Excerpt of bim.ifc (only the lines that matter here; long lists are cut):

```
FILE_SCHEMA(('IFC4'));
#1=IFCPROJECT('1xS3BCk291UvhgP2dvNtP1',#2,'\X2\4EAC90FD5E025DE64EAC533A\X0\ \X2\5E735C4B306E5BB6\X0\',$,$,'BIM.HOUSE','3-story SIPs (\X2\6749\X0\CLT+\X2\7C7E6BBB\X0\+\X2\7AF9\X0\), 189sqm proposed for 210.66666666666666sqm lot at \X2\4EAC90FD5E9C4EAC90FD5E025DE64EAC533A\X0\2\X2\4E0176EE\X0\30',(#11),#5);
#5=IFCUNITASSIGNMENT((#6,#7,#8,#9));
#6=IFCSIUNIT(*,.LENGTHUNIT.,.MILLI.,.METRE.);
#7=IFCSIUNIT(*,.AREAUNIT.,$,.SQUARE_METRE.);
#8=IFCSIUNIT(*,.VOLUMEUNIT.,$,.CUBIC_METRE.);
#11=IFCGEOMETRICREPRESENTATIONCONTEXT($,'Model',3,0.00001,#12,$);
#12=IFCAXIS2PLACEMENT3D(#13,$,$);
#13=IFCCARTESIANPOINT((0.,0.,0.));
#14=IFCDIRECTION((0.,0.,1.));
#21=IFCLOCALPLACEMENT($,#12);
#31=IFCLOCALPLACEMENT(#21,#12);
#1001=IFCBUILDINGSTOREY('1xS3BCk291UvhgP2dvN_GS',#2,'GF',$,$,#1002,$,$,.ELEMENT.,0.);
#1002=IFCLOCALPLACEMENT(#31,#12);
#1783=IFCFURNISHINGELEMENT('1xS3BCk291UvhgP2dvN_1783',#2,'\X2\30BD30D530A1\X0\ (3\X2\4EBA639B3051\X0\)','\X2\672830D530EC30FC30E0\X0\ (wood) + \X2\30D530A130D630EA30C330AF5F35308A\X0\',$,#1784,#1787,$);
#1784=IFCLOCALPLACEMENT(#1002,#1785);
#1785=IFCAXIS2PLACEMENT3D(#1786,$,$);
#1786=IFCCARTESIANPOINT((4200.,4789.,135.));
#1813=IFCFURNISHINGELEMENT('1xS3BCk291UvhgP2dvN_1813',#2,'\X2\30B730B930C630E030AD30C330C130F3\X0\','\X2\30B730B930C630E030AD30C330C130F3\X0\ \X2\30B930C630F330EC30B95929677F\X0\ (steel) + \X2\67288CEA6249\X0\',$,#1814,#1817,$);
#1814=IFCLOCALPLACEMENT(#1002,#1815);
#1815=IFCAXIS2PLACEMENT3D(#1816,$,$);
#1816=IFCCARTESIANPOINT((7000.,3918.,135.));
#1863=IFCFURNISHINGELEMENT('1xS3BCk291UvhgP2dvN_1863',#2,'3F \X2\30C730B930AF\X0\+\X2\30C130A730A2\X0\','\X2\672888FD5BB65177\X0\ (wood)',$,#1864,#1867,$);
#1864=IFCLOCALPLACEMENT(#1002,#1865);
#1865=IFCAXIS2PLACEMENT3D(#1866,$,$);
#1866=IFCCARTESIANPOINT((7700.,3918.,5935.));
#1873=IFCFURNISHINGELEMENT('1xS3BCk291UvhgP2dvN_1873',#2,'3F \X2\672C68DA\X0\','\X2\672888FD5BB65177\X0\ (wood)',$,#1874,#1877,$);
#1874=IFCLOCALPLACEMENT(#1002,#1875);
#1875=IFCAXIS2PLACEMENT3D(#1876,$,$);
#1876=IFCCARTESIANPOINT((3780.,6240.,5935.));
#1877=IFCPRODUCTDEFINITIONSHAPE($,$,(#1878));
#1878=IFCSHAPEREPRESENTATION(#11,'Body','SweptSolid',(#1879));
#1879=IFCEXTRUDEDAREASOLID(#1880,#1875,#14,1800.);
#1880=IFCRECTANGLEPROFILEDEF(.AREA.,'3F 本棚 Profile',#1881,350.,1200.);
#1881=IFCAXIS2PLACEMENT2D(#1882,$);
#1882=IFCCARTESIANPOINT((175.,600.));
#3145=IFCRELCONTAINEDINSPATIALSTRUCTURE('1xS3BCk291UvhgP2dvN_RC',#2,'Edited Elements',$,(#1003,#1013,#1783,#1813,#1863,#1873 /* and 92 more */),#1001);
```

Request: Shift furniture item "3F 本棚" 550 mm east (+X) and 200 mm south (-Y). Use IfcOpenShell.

```python
import ifcopenshell
import ifcopenshell.api.geometry
import ifcopenshell.util.placement
import ifcopenshell.util.unit

model = ifcopenshell.open("bim.ifc")
unit_scale = ifcopenshell.util.unit.calculate_unit_scale(model)

item = model.by_guid("1xS3BCk291UvhgP2dvN_1873")
matrix = ifcopenshell.util.placement.get_local_placement(item.ObjectPlacement)
matrix[0, 3] += 0.55 / unit_scale
matrix[1, 3] -= 0.2 / unit_scale
ifcopenshell.api.geometry.edit_object_placement(model, product=item, matrix=matrix, is_si=False)

print(ifcopenshell.util.placement.get_local_placement(item.ObjectPlacement).round(3) + 0.0)

model.write("bim_updated.ifc")
```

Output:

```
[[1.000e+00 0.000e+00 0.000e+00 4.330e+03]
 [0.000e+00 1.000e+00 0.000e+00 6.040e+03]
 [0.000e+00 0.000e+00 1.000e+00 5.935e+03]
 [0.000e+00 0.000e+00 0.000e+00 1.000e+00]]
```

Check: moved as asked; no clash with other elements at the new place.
